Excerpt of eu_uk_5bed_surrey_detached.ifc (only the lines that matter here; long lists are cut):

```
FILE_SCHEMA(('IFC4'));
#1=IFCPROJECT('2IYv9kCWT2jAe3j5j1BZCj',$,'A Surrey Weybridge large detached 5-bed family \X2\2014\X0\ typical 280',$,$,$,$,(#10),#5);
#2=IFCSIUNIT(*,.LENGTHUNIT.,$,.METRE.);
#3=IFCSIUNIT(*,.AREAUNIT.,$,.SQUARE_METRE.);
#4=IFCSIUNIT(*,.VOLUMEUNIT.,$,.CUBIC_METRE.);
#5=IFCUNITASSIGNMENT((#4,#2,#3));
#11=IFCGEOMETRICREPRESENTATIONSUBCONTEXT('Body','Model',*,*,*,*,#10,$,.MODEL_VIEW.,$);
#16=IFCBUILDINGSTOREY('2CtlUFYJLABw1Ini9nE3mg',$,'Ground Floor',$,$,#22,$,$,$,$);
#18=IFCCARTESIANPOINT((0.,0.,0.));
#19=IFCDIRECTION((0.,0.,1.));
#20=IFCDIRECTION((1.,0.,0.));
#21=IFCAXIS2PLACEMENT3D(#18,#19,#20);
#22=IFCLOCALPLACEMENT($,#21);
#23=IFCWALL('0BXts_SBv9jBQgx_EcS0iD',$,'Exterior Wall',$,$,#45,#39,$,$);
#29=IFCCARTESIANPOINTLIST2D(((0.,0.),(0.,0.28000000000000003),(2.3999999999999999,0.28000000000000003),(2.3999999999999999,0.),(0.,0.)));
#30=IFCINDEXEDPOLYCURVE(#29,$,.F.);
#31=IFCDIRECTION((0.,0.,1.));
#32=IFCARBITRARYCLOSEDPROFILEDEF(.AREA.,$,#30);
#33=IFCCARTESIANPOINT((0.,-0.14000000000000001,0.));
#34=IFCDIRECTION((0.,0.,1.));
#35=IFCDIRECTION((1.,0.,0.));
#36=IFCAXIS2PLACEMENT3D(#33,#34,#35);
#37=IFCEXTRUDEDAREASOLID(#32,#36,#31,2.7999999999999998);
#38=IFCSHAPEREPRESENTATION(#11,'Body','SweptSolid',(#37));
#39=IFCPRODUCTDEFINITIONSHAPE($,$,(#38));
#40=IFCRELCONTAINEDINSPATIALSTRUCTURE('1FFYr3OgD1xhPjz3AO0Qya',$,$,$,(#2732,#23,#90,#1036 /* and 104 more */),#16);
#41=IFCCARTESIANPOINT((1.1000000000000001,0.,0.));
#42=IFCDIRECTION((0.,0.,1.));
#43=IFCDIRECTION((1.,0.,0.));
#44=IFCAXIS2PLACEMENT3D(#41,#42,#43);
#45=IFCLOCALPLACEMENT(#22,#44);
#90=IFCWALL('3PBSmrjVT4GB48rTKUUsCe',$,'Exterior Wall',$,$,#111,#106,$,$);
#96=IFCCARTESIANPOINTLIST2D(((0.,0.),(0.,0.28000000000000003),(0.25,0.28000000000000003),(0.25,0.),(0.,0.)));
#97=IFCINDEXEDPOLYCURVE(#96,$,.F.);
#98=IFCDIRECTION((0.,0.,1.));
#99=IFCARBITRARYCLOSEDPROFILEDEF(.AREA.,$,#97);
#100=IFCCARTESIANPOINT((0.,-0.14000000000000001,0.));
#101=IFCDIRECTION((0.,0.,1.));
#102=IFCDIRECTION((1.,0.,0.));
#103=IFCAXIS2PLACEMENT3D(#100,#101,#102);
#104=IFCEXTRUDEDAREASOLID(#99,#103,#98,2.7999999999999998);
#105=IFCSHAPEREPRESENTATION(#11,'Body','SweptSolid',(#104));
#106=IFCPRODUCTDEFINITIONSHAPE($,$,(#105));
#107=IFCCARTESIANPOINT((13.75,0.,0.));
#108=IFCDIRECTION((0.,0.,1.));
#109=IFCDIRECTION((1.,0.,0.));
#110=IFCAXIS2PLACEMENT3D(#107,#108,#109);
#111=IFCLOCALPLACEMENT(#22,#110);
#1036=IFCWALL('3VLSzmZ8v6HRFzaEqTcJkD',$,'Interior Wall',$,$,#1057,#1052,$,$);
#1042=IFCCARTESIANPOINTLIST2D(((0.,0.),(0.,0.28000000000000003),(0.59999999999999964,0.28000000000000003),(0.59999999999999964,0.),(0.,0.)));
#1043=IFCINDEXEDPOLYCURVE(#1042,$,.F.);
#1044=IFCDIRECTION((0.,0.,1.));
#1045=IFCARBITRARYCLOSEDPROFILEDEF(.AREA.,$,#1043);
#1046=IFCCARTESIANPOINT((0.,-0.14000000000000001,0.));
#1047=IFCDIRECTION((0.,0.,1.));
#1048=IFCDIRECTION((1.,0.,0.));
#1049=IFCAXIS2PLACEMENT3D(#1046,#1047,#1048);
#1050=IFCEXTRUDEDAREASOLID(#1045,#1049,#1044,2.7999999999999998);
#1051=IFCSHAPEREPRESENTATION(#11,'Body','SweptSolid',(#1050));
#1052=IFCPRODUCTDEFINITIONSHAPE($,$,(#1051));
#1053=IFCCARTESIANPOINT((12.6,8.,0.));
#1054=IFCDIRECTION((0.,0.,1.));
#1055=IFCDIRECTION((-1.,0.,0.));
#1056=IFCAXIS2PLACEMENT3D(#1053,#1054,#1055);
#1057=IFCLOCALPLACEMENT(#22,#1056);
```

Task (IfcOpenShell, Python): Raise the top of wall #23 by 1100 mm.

```python
import ifcopenshell
import ifcopenshell.geom
import ifcopenshell.util.representation
import ifcopenshell.util.shape
import ifcopenshell.util.unit

model = ifcopenshell.open("eu_uk_5bed_surrey_detached.ifc")
unit_scale = ifcopenshell.util.unit.calculate_unit_scale(model)
settings = ifcopenshell.geom.settings()


def volume(element):
    """Net volume in cubic metres, openings subtracted."""
    shape = ifcopenshell.geom.create_shape(settings, element)
    return ifcopenshell.util.shape.get_volume(shape.geometry)


wall = model.by_id(23)
before = volume(wall)

body = ifcopenshell.util.representation.get_representation(wall, "Model", "Body")
solid = body.Items[0]
old_height = solid.Depth
solid.Depth += 1.1 / unit_scale
after = volume(wall)

print(f"height {old_height:g} -> {solid.Depth:g}, volume {before:.3f} -> {after:.3f} m3")

model.write("eu_uk_5bed_surrey_detached-out.ifc")
```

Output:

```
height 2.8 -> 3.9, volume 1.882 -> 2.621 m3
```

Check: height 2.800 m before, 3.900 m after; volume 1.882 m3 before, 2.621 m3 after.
